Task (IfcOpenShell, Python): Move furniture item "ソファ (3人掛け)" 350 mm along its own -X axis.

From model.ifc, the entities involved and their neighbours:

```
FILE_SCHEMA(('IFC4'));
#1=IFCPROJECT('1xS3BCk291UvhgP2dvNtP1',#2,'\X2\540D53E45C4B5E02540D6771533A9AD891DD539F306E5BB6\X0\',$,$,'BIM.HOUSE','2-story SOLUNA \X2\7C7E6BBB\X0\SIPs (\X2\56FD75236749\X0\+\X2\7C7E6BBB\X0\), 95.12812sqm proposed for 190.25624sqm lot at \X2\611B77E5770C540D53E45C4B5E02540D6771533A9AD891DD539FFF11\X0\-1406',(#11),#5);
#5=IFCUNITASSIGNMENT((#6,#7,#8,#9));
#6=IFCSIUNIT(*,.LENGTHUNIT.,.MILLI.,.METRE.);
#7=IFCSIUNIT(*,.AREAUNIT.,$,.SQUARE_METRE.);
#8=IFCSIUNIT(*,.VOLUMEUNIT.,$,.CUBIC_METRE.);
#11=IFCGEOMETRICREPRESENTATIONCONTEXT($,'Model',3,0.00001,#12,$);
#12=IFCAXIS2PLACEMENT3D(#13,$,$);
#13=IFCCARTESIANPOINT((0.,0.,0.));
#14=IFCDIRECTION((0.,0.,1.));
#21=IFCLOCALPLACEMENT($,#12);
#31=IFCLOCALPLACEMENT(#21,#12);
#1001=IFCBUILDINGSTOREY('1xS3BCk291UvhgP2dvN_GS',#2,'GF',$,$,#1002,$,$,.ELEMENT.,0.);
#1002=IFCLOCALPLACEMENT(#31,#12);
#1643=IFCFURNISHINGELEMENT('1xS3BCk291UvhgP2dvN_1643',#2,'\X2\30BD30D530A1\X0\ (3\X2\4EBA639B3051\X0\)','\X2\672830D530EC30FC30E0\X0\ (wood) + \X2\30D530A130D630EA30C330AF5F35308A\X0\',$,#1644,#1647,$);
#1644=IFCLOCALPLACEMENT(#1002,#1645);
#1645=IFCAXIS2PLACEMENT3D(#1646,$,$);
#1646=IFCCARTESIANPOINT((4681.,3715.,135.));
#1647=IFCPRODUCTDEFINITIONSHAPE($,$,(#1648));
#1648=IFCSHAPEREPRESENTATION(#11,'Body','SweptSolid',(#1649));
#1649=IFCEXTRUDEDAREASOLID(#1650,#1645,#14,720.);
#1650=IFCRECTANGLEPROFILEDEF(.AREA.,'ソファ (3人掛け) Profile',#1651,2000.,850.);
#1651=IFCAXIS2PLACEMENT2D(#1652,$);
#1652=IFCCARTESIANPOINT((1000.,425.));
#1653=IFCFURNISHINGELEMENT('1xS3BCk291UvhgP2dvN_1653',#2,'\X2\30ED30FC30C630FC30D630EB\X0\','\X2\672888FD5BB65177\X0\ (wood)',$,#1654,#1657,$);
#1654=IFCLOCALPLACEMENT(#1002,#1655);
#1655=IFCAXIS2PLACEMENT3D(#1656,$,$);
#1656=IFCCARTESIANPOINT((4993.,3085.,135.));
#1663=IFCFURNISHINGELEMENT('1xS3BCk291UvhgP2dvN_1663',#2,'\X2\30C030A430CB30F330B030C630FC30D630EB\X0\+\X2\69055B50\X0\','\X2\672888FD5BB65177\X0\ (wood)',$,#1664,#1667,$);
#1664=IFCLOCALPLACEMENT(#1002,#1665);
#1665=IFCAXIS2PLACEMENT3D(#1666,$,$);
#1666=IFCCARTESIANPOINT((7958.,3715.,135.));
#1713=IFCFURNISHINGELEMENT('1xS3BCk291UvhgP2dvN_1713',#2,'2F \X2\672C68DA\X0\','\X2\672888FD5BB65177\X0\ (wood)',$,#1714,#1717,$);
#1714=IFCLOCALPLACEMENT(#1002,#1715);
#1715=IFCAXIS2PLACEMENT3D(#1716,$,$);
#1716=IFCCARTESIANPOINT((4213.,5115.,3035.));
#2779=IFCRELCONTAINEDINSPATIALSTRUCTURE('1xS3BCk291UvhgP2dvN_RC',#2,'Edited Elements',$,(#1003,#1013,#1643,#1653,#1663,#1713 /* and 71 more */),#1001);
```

```python
import ifcopenshell
import ifcopenshell.api.geometry
import ifcopenshell.util.placement
import ifcopenshell.util.unit

model = ifcopenshell.open("model.ifc")
unit_scale = ifcopenshell.util.unit.calculate_unit_scale(model)

item = model.by_guid("1xS3BCk291UvhgP2dvN_1643")
matrix = ifcopenshell.util.placement.get_local_placement(item.ObjectPlacement)
matrix[:3, 3] -= matrix[:3, 0] * 0.35 / unit_scale
ifcopenshell.api.geometry.edit_object_placement(model, product=item, matrix=matrix, is_si=False)

print(ifcopenshell.util.placement.get_local_placement(item.ObjectPlacement).round(3) + 0.0)

model.write("model_updated.ifc")
```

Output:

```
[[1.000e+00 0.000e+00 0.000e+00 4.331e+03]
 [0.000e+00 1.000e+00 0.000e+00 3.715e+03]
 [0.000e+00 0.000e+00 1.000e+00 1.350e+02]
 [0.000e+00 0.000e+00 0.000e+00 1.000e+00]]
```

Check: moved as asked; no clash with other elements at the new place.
